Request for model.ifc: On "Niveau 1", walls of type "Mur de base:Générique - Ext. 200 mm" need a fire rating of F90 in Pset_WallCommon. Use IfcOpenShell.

First a look at what the model holds.

```python
import ifcopenshell
import ifcopenshell.util.element

model = ifcopenshell.open("model.ifc")
print(model.schema)
storey = next(s for s in model.by_type("IfcBuildingStorey") if s.Name == "Niveau 1")
walls = [e for e in ifcopenshell.util.element.get_decomposition(storey) if e.is_a("IfcWall")]
seen = {}
for e in walls:
    element_type = ifcopenshell.util.element.get_type(e)
    key = (element_type.Name if element_type != e and element_type else None, ifcopenshell.util.element.get_pset(e, "Pset_WallCommon", "FireRating"))
    seen[key] = seen.get(key, 0) + 1
for (name, value), count in sorted(seen.items(), key=str):
    print(count, "x", name, "|", value)
```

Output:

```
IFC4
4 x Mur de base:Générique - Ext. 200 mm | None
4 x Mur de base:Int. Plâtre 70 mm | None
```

```python
import ifcopenshell
import ifcopenshell.api.pset
import ifcopenshell.util.element

model = ifcopenshell.open("model.ifc")

storey = next(s for s in model.by_type("IfcBuildingStorey") if s.Name == "Niveau 1")
walls = [e for e in ifcopenshell.util.element.get_decomposition(storey) if e.is_a("IfcWall")]

count = 0
for e in walls:
    element_type = ifcopenshell.util.element.get_type(e)
    if element_type in (None, e) or element_type.Name != "Mur de base:Générique - Ext. 200 mm":
        continue
    # add_pset returns the element's existing set when there is one.
    pset = ifcopenshell.api.pset.add_pset(model, product=e, name="Pset_WallCommon")
    ifcopenshell.api.pset.edit_pset(model, pset=pset, properties={"FireRating": "F90"})
    count += 1

print(count, "walls updated")

model.write("model_updated.ifc")
```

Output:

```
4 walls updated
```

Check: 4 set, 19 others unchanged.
